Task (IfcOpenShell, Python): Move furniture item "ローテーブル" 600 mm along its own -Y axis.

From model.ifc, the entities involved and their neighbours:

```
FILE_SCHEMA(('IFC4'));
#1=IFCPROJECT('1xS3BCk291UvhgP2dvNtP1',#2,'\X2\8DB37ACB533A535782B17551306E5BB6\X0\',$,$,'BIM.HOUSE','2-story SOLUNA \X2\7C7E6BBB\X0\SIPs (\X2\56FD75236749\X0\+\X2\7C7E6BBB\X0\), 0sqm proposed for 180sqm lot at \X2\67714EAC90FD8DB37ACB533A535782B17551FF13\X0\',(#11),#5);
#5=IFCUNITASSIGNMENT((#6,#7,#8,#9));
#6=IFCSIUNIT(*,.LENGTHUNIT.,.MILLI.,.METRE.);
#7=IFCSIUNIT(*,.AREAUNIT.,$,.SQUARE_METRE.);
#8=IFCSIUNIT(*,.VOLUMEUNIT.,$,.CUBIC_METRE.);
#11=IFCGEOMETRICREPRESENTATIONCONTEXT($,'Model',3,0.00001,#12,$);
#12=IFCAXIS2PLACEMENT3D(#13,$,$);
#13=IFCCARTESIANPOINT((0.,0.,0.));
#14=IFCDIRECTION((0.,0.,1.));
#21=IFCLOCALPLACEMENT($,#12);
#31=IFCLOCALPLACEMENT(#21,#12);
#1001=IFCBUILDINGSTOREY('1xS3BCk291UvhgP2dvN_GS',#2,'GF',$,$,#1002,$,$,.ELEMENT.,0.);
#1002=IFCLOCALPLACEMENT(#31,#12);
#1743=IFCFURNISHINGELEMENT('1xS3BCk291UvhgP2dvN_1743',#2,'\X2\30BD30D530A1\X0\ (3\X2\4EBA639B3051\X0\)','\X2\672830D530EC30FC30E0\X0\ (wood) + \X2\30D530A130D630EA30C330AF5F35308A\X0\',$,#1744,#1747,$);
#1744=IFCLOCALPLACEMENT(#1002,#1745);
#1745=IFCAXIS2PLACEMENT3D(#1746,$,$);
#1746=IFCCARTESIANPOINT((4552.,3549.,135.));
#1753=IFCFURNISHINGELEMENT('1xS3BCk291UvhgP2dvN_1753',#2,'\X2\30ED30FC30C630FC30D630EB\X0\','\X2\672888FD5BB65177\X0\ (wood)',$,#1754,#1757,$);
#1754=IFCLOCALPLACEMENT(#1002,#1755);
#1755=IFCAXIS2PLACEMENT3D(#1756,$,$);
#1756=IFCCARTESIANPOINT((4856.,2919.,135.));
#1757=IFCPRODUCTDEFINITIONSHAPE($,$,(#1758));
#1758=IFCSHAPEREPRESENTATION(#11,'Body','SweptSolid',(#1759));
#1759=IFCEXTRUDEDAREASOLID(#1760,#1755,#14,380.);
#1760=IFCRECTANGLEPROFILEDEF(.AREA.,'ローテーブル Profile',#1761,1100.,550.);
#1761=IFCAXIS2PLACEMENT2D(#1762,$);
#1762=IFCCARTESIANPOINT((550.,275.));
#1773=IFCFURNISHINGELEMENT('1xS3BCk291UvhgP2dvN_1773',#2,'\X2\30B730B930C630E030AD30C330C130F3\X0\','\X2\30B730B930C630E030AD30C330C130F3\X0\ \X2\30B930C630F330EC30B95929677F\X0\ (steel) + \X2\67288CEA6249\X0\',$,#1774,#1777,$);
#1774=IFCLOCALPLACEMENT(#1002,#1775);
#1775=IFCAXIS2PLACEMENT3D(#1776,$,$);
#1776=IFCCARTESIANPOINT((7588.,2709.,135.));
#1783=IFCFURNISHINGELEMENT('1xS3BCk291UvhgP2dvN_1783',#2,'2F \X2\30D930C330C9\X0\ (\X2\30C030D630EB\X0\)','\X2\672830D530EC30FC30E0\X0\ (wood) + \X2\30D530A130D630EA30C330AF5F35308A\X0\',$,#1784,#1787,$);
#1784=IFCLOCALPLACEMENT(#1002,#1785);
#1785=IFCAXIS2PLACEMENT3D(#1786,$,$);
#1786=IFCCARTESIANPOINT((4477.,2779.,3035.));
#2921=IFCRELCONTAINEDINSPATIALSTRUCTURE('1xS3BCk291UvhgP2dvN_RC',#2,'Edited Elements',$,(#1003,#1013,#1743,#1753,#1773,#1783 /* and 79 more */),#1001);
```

```python
import ifcopenshell
import ifcopenshell.api.geometry
import ifcopenshell.util.placement
import ifcopenshell.util.unit

model = ifcopenshell.open("model.ifc")
unit_scale = ifcopenshell.util.unit.calculate_unit_scale(model)

item = model.by_guid("1xS3BCk291UvhgP2dvN_1753")
matrix = ifcopenshell.util.placement.get_local_placement(item.ObjectPlacement)
matrix[:3, 3] -= matrix[:3, 1] * 0.6 / unit_scale
ifcopenshell.api.geometry.edit_object_placement(model, product=item, matrix=matrix, is_si=False)

print(ifcopenshell.util.placement.get_local_placement(item.ObjectPlacement).round(3) + 0.0)

model.write("model_v2.ifc")
```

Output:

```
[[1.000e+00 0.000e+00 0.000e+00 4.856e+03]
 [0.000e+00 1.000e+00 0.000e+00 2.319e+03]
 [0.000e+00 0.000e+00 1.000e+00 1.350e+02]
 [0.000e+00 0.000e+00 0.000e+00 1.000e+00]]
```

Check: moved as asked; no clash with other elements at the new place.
